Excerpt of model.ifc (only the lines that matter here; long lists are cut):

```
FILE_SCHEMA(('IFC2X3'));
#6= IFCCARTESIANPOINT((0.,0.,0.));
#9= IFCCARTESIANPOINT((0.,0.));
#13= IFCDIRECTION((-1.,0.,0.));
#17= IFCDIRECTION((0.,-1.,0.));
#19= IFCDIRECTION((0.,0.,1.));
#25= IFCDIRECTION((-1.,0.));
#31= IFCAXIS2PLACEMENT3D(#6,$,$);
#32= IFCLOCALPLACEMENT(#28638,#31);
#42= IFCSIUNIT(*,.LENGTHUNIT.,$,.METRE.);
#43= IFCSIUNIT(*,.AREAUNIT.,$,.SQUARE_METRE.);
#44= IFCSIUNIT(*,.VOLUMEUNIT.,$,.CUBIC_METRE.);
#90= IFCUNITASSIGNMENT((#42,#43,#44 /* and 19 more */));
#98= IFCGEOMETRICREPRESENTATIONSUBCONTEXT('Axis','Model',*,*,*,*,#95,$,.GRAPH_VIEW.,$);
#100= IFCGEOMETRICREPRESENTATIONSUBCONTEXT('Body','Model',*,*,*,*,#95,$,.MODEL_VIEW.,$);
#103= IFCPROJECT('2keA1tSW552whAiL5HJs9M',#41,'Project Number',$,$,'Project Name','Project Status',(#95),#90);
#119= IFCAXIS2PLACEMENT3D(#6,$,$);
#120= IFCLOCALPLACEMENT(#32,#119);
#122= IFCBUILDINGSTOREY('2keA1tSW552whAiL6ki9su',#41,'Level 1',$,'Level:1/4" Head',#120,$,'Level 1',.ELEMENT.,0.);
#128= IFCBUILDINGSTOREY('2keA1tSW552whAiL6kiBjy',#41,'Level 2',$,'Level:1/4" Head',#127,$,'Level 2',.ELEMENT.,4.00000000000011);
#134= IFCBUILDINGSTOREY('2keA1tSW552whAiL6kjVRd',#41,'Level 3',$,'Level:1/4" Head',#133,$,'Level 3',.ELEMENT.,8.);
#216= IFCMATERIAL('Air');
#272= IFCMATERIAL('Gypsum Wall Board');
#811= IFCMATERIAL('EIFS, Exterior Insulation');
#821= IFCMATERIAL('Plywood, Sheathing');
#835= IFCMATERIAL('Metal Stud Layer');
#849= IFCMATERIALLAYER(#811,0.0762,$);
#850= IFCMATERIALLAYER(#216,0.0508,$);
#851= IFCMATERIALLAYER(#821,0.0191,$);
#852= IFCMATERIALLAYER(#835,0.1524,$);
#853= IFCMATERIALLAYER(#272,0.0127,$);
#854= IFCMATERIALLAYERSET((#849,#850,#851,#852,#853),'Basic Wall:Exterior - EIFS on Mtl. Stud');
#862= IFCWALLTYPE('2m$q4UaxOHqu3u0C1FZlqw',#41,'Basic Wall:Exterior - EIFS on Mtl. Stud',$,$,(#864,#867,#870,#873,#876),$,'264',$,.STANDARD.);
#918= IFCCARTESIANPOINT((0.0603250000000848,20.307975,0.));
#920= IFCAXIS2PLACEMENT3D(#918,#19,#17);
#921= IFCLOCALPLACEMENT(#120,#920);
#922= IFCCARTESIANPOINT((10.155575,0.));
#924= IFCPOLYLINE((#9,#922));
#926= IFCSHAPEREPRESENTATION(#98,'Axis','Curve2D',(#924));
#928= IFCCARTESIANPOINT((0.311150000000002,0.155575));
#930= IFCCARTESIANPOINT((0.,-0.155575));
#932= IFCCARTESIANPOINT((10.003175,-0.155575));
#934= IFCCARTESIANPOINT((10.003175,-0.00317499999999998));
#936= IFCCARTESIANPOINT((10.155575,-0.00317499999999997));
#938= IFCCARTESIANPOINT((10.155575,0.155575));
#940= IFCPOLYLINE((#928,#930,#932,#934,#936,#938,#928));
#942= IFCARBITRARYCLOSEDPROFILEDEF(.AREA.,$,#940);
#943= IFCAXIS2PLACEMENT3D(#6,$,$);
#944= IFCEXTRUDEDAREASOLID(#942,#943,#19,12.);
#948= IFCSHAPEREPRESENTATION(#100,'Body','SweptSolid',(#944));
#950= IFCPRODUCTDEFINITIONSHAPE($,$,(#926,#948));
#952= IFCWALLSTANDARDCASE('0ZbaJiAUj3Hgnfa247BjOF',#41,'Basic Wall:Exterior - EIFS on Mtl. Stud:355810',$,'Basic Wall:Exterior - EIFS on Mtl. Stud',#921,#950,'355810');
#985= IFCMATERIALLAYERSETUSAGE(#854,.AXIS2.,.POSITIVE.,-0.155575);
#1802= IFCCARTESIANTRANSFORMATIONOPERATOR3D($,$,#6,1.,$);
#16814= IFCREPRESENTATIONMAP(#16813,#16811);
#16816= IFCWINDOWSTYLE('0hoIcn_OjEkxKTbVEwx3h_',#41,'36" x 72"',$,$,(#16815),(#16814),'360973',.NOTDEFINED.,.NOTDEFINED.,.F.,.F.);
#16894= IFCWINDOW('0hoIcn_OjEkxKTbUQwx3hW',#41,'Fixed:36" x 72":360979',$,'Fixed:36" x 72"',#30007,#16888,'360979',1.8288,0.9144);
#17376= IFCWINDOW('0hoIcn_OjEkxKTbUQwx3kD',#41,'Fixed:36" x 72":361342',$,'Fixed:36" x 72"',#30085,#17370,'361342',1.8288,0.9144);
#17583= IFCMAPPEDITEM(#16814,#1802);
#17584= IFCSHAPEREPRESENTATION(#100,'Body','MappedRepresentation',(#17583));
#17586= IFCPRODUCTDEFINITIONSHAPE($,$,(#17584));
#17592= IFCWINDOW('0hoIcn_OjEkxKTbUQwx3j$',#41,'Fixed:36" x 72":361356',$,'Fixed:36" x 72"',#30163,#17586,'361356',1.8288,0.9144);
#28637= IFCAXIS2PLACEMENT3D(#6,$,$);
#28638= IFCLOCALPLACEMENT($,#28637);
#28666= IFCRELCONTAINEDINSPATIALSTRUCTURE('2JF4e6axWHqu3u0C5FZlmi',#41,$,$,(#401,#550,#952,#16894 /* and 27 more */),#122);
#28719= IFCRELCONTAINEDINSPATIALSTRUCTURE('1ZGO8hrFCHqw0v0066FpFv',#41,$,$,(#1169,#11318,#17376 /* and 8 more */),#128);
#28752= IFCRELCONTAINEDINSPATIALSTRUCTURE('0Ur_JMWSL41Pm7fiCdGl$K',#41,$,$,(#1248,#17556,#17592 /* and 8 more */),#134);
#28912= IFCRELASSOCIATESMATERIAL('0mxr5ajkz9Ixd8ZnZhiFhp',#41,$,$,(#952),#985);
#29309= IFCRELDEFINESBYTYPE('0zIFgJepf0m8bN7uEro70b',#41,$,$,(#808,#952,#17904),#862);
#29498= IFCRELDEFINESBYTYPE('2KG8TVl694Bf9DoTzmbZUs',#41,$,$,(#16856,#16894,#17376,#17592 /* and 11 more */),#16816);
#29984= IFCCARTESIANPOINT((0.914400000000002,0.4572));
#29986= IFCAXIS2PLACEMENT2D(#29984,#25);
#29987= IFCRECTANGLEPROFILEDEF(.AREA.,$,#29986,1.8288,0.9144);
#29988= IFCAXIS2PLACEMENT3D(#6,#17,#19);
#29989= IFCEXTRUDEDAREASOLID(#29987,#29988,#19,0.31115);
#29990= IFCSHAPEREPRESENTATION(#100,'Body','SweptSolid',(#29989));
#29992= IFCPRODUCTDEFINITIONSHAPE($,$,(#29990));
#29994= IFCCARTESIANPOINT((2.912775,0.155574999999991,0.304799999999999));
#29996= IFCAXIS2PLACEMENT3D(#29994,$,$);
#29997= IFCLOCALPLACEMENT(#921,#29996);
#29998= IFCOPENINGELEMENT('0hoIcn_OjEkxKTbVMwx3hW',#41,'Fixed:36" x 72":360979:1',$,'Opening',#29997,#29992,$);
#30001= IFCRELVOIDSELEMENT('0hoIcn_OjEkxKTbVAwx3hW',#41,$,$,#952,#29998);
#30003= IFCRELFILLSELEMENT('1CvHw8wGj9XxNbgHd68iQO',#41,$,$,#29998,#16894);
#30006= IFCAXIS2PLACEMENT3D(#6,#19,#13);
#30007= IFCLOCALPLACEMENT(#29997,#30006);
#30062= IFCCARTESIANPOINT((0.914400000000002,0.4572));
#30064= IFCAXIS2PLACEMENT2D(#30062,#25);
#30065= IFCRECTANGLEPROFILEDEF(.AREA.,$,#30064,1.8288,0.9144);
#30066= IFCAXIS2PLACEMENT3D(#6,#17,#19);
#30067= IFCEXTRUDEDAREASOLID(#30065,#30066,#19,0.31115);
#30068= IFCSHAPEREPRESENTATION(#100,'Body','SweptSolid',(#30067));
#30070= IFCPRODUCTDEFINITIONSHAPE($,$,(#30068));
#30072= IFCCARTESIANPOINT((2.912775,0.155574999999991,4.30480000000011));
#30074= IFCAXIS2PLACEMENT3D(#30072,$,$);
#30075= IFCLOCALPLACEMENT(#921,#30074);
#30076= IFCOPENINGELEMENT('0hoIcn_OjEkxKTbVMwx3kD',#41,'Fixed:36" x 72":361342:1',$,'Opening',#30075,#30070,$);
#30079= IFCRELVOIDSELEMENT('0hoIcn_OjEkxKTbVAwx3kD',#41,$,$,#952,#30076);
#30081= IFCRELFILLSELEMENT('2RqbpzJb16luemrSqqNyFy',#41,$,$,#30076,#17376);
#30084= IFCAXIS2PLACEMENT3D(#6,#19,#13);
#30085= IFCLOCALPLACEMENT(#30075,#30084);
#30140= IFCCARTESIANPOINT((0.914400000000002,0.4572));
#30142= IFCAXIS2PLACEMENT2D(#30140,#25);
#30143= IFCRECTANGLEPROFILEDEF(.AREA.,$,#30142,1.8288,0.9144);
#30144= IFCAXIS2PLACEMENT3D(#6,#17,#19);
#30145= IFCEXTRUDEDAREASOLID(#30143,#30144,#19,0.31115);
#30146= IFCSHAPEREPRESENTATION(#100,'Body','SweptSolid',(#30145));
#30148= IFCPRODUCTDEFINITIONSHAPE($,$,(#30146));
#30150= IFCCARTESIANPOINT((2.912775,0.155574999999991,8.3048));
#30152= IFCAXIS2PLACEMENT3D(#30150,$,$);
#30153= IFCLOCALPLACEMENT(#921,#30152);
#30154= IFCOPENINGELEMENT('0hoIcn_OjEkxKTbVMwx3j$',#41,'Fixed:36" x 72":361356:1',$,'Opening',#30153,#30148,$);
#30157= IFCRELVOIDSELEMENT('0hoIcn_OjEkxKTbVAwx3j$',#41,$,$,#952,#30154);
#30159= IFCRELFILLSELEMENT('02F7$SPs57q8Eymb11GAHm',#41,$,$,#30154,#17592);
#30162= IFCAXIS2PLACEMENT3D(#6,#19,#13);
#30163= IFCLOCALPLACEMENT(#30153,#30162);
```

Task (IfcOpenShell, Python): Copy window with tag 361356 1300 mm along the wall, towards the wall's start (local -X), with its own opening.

```python
import ifcopenshell
import ifcopenshell.api.feature
import ifcopenshell.api.geometry
import ifcopenshell.api.root
import ifcopenshell.geom
import ifcopenshell.util.element
import ifcopenshell.util.placement
import ifcopenshell.util.shape

model = ifcopenshell.open("model.ifc")
settings = ifcopenshell.geom.settings()


def volume(element):
    """Net volume in cubic metres, openings subtracted."""
    shape = ifcopenshell.geom.create_shape(settings, element)
    return ifcopenshell.util.shape.get_volume(shape.geometry)


def reuse_history(source, copy):
    """copy_class also copies each property set's owner history, people and application; keep the originals."""
    for rel in copy.IsDefinedBy:
        if rel.is_a("IfcRelDefinesByProperties") and (history := rel.RelatingPropertyDefinition.OwnerHistory):
            rel.RelatingPropertyDefinition.OwnerHistory = source.OwnerHistory
            ifcopenshell.util.element.remove_deep2(model, history)


window = model.by_guid("0hoIcn_OjEkxKTbUQwx3j$")
opening = window.FillsVoids[0].RelatingOpeningElement
wall = opening.VoidsElements[0].RelatingBuildingElement
before = volume(wall)
shift = ifcopenshell.util.placement.get_local_placement(wall.ObjectPlacement)[:3, 0] * -1.3

# copy_class copies the void relationship, type, container and properties, but no geometry.
new_opening = ifcopenshell.api.root.copy_class(model, product=opening)
new_opening.Representation = ifcopenshell.util.element.copy_deep(
    model, opening.Representation, exclude=["IfcGeometricRepresentationContext", "IfcRepresentationMap"]
)
new_opening.Name = 'Fixed:36" x 72"'
new_window = ifcopenshell.api.root.copy_class(model, product=window)
new_window.Representation = ifcopenshell.util.element.copy_deep(
    model, window.Representation, exclude=["IfcGeometricRepresentationContext", "IfcRepresentationMap"]
)
new_window.Name = 'Fixed:36" x 72"'
new_window.Tag = None
reuse_history(window, new_window)
fills = ifcopenshell.api.feature.add_filling(model, opening=new_opening, element=new_window)
fills.OwnerHistory = new_window.OwnerHistory  # required in IFC2X3

for old, new in ((opening, new_opening), (window, new_window)):
    matrix = ifcopenshell.util.placement.get_local_placement(old.ObjectPlacement)
    matrix[:3, 3] += shift
    ifcopenshell.api.geometry.edit_object_placement(model, product=new, matrix=matrix, is_si=False)

after = volume(wall)

print(f"wall volume {before:.3f} -> {after:.3f} m3")

model.write("model-out.ifc")
```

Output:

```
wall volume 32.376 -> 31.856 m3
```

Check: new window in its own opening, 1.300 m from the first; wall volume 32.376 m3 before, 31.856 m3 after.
